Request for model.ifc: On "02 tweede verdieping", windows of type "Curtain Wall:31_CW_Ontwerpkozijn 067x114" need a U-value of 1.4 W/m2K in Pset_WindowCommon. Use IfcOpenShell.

First a look at what the model holds.

```python
import ifcopenshell
import ifcopenshell.util.element

model = ifcopenshell.open("model.ifc")
print(model.schema)
storey = next(s for s in model.by_type("IfcBuildingStorey") if s.Name == "02 tweede verdieping")
windows = [e for e in ifcopenshell.util.element.get_decomposition(storey) if e.is_a("IfcWindow")]
seen = {}
for e in windows:
    element_type = ifcopenshell.util.element.get_type(e)
    key = (element_type.Name if element_type != e and element_type else None, ifcopenshell.util.element.get_pset(e, "Pset_WindowCommon", "ThermalTransmittance"))
    seen[key] = seen.get(key, 0) + 1
for (name, value), count in sorted(seen.items(), key=str):
    print(count, "x", name, "|", value)
```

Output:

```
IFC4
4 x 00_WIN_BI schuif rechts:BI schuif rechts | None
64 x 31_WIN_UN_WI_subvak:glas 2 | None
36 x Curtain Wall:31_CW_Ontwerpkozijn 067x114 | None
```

```python
import ifcopenshell
import ifcopenshell.api.pset
import ifcopenshell.util.element

model = ifcopenshell.open("model.ifc")

storey = next(s for s in model.by_type("IfcBuildingStorey") if s.Name == "02 tweede verdieping")
windows = [e for e in ifcopenshell.util.element.get_decomposition(storey) if e.is_a("IfcWindow")]

count = 0
for e in windows:
    element_type = ifcopenshell.util.element.get_type(e)
    if element_type in (None, e) or element_type.Name != "Curtain Wall:31_CW_Ontwerpkozijn 067x114":
        continue
    # add_pset returns the element's existing set when there is one.
    pset = ifcopenshell.api.pset.add_pset(model, product=e, name="Pset_WindowCommon")
    ifcopenshell.api.pset.edit_pset(model, pset=pset, properties={"ThermalTransmittance": 1.4})
    count += 1

print(count, "windows updated")

model.write("model_v2.ifc")
```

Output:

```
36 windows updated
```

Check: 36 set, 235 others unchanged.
